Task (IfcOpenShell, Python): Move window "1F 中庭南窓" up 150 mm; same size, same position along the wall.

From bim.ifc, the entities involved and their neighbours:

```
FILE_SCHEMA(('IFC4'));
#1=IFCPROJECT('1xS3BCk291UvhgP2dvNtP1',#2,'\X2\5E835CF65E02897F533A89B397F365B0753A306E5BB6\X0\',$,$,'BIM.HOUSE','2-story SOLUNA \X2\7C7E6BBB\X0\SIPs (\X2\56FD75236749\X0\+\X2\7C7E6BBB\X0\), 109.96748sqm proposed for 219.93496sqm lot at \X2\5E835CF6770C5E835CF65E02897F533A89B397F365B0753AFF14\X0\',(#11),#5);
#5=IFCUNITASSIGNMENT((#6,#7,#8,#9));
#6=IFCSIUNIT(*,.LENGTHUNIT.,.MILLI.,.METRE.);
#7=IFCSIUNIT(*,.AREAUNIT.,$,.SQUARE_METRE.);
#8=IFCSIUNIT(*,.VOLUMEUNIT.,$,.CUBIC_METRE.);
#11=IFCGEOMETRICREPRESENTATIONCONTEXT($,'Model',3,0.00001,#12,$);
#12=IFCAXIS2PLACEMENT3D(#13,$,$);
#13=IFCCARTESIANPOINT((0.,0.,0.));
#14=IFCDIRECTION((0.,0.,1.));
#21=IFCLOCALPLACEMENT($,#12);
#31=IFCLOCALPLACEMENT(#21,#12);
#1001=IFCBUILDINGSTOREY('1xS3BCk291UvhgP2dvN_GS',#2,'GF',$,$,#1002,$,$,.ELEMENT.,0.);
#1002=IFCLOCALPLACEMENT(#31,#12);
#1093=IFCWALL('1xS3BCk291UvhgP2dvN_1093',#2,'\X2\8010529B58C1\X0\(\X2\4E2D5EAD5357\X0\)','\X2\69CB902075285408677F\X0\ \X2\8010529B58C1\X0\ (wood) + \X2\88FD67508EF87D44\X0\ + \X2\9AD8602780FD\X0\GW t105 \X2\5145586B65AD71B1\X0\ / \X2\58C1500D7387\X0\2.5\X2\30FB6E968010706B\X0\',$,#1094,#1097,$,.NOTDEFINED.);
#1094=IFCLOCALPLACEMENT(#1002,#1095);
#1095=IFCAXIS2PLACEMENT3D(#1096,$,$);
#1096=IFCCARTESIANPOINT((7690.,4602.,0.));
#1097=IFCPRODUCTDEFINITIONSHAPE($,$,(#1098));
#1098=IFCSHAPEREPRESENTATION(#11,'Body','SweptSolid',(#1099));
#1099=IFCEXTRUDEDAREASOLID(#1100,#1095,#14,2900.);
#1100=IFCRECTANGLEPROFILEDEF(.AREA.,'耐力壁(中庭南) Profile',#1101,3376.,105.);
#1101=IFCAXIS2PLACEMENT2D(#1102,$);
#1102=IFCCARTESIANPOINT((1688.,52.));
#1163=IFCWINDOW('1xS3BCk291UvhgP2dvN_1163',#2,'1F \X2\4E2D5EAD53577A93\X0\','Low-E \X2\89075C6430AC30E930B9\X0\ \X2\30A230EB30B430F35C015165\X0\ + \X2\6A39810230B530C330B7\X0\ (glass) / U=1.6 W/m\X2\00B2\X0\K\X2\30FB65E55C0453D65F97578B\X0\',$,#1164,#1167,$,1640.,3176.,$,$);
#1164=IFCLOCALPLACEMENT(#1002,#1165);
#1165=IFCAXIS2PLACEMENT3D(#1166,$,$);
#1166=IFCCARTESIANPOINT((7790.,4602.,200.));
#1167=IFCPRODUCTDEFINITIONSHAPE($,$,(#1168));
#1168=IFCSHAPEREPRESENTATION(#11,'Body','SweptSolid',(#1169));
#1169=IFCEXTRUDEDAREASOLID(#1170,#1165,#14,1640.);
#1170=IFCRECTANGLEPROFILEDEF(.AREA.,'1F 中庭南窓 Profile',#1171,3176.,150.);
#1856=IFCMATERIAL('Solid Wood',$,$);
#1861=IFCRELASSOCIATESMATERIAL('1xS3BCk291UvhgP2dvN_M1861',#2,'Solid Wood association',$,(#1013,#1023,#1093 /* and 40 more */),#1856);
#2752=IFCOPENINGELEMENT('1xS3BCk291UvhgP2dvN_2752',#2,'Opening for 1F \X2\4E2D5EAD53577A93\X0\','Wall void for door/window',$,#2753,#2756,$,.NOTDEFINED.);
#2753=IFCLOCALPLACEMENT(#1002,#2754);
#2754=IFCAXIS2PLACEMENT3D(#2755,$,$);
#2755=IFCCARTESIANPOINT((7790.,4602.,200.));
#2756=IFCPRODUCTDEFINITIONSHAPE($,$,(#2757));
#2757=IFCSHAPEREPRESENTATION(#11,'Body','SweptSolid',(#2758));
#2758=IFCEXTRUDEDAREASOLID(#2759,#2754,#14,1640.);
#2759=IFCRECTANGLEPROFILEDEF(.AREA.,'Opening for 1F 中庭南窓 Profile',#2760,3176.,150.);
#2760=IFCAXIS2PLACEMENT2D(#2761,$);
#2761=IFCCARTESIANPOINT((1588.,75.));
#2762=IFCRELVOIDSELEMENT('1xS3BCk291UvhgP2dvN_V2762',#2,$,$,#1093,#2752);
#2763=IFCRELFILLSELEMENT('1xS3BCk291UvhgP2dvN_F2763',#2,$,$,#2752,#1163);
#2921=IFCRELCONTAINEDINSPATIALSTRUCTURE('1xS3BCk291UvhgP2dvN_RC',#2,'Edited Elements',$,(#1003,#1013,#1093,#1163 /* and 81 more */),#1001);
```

```python
import numpy as np
import ifcopenshell
import ifcopenshell.api.geometry
import ifcopenshell.util.placement
import ifcopenshell.util.unit

model = ifcopenshell.open("bim.ifc")
unit_scale = ifcopenshell.util.unit.calculate_unit_scale(model)

window = model.by_id(1163)
opening = window.FillsVoids[0].RelatingOpeningElement
dz = 150.0

shift = np.array([0.0, 0.0, dz])
# The window is not placed relative to its opening, so move both.
for product in (opening, window):
    matrix = ifcopenshell.util.placement.get_local_placement(product.ObjectPlacement)
    matrix[:3, 3] += shift
    ifcopenshell.api.geometry.edit_object_placement(model, product=product, matrix=matrix, is_si=False)

print(f"moved by {dz * unit_scale:+.3f} m")

model.write("bim_edited.ifc")
```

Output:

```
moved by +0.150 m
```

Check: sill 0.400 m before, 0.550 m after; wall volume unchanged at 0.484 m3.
